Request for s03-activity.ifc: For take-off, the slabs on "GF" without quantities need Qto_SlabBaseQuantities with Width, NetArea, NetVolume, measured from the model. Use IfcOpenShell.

First a look at what the model holds.

```python
import ifcopenshell
import ifcopenshell.util.element
import ifcopenshell.util.unit

model = ifcopenshell.open("s03-activity.ifc")
print(model.schema)
for unit_type in ("LENGTHUNIT", "AREAUNIT", "VOLUMEUNIT"):
    print(unit_type, ifcopenshell.util.unit.calculate_unit_scale(model, unit_type))
storey = next(s for s in model.by_type("IfcBuildingStorey") if s.Name == "GF")
slabs = [e for e in ifcopenshell.util.element.get_decomposition(storey) if e.is_a("IfcSlab")]
for e in sorted(slabs, key=lambda e: e.id()):
    print(e.id(), e.is_a(), e.Name, list(ifcopenshell.util.element.get_psets(e, qtos_only=True)), sep=" | ")
```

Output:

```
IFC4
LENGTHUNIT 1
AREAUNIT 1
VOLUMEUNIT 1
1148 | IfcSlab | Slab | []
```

```python
import ifcopenshell
import ifcopenshell.api.pset
import ifcopenshell.geom
import ifcopenshell.util.element
import ifcopenshell.util.shape
import ifcopenshell.util.unit

model = ifcopenshell.open("s03-activity.ifc")
unit_scale = ifcopenshell.util.unit.calculate_unit_scale(model)
area_scale = ifcopenshell.util.unit.calculate_unit_scale(model, "AREAUNIT")
volume_scale = ifcopenshell.util.unit.calculate_unit_scale(model, "VOLUMEUNIT")
settings = ifcopenshell.geom.settings()

storey = next(s for s in model.by_type("IfcBuildingStorey") if s.Name == "GF")
slabs = [e for e in ifcopenshell.util.element.get_decomposition(storey) if e.is_a("IfcSlab")]

for e in sorted(slabs, key=lambda e: e.id()):
    if ifcopenshell.util.element.get_psets(e, qtos_only=True, should_inherit=False):
        continue
    # Geometry comes back in metres, in the element's own axes.
    shape = ifcopenshell.geom.create_shape(settings, e)
    values = {
        "Width": ifcopenshell.util.shape.get_z(shape.geometry) / unit_scale,
        "NetArea": ifcopenshell.util.shape.get_footprint_area(shape.geometry) / area_scale,
        "NetVolume": ifcopenshell.util.shape.get_volume(shape.geometry) / volume_scale,
    }
    qto = ifcopenshell.api.pset.add_qto(model, product=e, name="Qto_SlabBaseQuantities")
    ifcopenshell.api.pset.edit_qto(model, qto=qto, properties=values)
    print(e.id(), {k: round(v, 3) for k, v in values.items()})

model.write("s03-activity_edited.ifc")
```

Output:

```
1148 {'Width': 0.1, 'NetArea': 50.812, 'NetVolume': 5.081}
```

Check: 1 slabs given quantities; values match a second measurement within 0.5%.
